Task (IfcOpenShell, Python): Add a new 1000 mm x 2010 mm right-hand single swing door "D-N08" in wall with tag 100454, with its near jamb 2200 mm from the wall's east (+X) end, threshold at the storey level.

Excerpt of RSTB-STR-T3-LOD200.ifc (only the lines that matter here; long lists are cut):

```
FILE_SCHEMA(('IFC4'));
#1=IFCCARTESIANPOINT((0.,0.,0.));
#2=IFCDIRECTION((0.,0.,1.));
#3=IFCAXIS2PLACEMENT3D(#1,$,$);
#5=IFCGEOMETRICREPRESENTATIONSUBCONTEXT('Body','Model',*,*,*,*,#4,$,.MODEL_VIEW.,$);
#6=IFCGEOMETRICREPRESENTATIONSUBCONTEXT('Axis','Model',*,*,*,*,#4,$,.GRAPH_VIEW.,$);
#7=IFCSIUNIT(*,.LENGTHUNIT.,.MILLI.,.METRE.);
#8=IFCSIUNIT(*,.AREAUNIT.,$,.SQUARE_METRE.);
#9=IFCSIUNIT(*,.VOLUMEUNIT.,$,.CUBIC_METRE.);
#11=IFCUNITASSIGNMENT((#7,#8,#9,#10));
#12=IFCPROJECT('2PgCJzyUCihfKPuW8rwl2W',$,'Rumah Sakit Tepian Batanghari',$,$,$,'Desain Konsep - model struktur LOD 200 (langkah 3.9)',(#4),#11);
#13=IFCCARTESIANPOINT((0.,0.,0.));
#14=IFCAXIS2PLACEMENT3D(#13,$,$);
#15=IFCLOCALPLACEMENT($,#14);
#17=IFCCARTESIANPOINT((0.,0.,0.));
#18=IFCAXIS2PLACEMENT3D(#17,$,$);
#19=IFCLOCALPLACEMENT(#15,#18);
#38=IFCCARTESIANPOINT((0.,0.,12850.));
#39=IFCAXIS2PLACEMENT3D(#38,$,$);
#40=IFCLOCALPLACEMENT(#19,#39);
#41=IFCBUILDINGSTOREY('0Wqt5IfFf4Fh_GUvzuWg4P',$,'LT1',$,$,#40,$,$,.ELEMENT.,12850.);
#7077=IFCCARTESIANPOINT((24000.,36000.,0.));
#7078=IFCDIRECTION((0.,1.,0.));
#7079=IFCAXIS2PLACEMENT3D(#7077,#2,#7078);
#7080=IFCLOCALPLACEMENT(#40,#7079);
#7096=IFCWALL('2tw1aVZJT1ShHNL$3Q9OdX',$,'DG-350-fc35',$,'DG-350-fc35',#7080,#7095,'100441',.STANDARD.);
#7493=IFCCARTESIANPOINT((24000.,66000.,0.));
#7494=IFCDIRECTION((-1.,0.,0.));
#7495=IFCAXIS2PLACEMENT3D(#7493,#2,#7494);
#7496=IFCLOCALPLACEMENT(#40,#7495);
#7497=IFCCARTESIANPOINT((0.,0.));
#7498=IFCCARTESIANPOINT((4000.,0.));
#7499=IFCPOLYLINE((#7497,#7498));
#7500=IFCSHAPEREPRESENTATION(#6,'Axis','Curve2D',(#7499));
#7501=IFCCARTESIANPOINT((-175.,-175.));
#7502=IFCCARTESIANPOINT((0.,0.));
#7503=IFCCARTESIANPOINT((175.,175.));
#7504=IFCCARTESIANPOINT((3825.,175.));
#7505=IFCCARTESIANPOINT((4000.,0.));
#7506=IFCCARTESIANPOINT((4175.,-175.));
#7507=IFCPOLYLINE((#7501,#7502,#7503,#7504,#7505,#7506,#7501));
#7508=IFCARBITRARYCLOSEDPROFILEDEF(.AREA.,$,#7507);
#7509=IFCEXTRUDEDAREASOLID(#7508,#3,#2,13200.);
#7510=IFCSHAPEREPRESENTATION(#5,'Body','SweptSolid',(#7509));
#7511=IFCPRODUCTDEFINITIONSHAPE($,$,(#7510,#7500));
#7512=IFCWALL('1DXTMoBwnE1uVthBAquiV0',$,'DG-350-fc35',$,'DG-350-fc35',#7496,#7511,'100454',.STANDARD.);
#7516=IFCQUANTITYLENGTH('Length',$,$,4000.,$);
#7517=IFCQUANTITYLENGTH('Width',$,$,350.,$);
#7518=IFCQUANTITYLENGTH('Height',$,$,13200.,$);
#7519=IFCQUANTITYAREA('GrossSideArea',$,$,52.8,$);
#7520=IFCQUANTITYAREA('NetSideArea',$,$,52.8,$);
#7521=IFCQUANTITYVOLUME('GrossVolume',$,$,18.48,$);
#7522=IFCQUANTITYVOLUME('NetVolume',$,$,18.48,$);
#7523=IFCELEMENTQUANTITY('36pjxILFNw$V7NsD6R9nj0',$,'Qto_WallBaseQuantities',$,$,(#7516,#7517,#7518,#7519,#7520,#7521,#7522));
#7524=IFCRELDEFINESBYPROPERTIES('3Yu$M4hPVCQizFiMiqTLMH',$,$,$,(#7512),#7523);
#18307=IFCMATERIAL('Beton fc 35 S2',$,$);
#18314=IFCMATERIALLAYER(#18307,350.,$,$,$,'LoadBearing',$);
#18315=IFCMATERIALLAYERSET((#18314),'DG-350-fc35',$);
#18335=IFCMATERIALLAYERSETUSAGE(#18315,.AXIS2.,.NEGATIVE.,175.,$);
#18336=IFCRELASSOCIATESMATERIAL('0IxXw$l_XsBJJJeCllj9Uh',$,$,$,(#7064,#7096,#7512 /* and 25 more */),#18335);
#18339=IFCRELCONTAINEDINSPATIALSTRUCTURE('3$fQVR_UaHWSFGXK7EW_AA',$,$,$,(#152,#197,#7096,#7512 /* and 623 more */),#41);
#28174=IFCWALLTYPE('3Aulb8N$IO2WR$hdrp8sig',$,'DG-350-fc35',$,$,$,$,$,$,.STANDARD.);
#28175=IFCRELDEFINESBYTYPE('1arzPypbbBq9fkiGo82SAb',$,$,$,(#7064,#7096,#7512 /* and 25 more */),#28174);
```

```python
import numpy as np
import ifcopenshell
import ifcopenshell.api.feature
import ifcopenshell.api.geometry
import ifcopenshell.api.pset
import ifcopenshell.api.root
import ifcopenshell.api.spatial
import ifcopenshell.geom
import ifcopenshell.util.element
import ifcopenshell.util.placement
import ifcopenshell.util.representation
import ifcopenshell.util.shape
import ifcopenshell.util.unit

model = ifcopenshell.open("RSTB-STR-T3-LOD200.ifc")
unit_scale = ifcopenshell.util.unit.calculate_unit_scale(model)
area_scale = ifcopenshell.util.unit.calculate_unit_scale(model, "AREAUNIT")
volume_scale = ifcopenshell.util.unit.calculate_unit_scale(model, "VOLUMEUNIT")
settings = ifcopenshell.geom.settings()


def volume(element):
    """Net volume in cubic metres, openings subtracted."""
    shape = ifcopenshell.geom.create_shape(settings, element)
    return ifcopenshell.util.shape.get_volume(shape.geometry)


wall = model.by_guid("1DXTMoBwnE1uVthBAquiV0")
storey = ifcopenshell.util.element.get_container(wall, ifc_class="IfcBuildingStorey")
context = ifcopenshell.util.representation.get_context(model, "Model", "Body", "MODEL_VIEW")
before = volume(wall)

width, height, from_end, sill = 1, 2.01, 2.2, 0.0  # metres

# The wall runs along its own X axis, and the end named is its -X end.
wall_shape = ifcopenshell.geom.create_shape(settings, wall)
x, y, z = ifcopenshell.util.shape.get_vertices(wall_shape.geometry).T
start = x.min() + from_end
face, thickness = float(y.min()), float(y.max() - y.min())
wall_matrix = ifcopenshell.util.placement.get_local_placement(wall.ObjectPlacement)
level = ifcopenshell.util.placement.get_local_placement(storey.ObjectPlacement)[2, 3]


def in_wall(x, y):
    """Placement at x, y metres in the wall's axes, at sill height."""
    matrix = wall_matrix.copy()
    matrix[:, 3] = wall_matrix @ np.array([x / unit_scale, y / unit_scale, 0.0, 1.0])
    matrix[2, 3] = level + sill / unit_scale
    return matrix


# Opening: a box that overshoots both wall faces by 50 mm.
opening = ifcopenshell.api.root.create_entity(model, ifc_class="IfcOpeningElement", predefined_type="OPENING")
box = ifcopenshell.api.geometry.add_wall_representation(
    model, context=context, length=width, height=height, thickness=thickness + 0.1
)
ifcopenshell.api.geometry.assign_representation(model, product=opening, representation=box)
ifcopenshell.api.geometry.edit_object_placement(model, product=opening, matrix=in_wall(start, face - 0.05), is_si=False)
ifcopenshell.api.feature.add_feature(model, feature=opening, element=wall)

door = ifcopenshell.api.root.create_entity(model, ifc_class="IfcDoor", name="D-N08", predefined_type="DOOR")
door.OverallWidth, door.OverallHeight = width / unit_scale, height / unit_scale
door.OperationType = "SINGLE_SWING_RIGHT"
body = ifcopenshell.api.geometry.add_door_representation(
    model,
    context=context,
    overall_width=door.OverallWidth,
    overall_height=door.OverallHeight,
    operation_type="SINGLE_SWING_RIGHT",
    lining_properties={"LiningDepth": thickness / unit_scale, "ThresholdDepth": thickness / unit_scale},
)
ifcopenshell.api.geometry.assign_representation(model, product=door, representation=body)
ifcopenshell.api.spatial.assign_container(model, products=[door], relating_structure=storey)
ifcopenshell.api.feature.add_filling(model, opening=opening, element=door)

# The lining spans the wall, so the door starts at the wall face.
ifcopenshell.api.geometry.edit_object_placement(model, product=door, matrix=in_wall(start, face), is_si=False)

after = volume(wall)

# Update the wall's stored quantities.
qto = model.by_id(ifcopenshell.util.element.get_pset(wall, "Qto_WallBaseQuantities", should_inherit=False)["id"])
ifcopenshell.api.pset.edit_qto(model, qto=qto, properties={
    "NetSideArea": after / thickness / area_scale,
    "NetVolume": after / volume_scale,
})

print(f"wall volume {before:.3f} -> {after:.3f} m3")

model.write("RSTB-STR-T3-LOD200_updated.ifc")
```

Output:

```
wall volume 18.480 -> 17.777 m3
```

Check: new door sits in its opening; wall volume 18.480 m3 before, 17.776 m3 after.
